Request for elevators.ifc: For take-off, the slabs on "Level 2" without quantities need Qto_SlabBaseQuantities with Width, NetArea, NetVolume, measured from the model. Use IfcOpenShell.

First a look at what the model holds.

```python
import ifcopenshell
import ifcopenshell.util.element
import ifcopenshell.util.unit

model = ifcopenshell.open("elevators.ifc")
print(model.schema)
for unit_type in ("LENGTHUNIT", "AREAUNIT", "VOLUMEUNIT"):
    print(unit_type, ifcopenshell.util.unit.calculate_unit_scale(model, unit_type))
storey = next(s for s in model.by_type("IfcBuildingStorey") if s.Name == "Level 2")
slabs = [e for e in ifcopenshell.util.element.get_decomposition(storey) if e.is_a("IfcSlab")]
for e in sorted(slabs, key=lambda e: e.id()):
    print(e.id(), e.is_a(), e.Name, list(ifcopenshell.util.element.get_psets(e, qtos_only=True)), sep=" | ")
```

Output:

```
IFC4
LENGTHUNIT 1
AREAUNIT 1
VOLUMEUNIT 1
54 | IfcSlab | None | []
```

```python
import ifcopenshell
import ifcopenshell.api.pset
import ifcopenshell.geom
import ifcopenshell.util.element
import ifcopenshell.util.shape
import ifcopenshell.util.unit

model = ifcopenshell.open("elevators.ifc")
unit_scale = ifcopenshell.util.unit.calculate_unit_scale(model)
area_scale = ifcopenshell.util.unit.calculate_unit_scale(model, "AREAUNIT")
volume_scale = ifcopenshell.util.unit.calculate_unit_scale(model, "VOLUMEUNIT")
settings = ifcopenshell.geom.settings()

storey = next(s for s in model.by_type("IfcBuildingStorey") if s.Name == "Level 2")
slabs = [e for e in ifcopenshell.util.element.get_decomposition(storey) if e.is_a("IfcSlab")]

for e in sorted(slabs, key=lambda e: e.id()):
    if ifcopenshell.util.element.get_psets(e, qtos_only=True, should_inherit=False):
        continue
    # Geometry comes back in metres, in the element's own axes.
    shape = ifcopenshell.geom.create_shape(settings, e)
    values = {
        "Width": ifcopenshell.util.shape.get_z(shape.geometry) / unit_scale,
        "NetArea": ifcopenshell.util.shape.get_footprint_area(shape.geometry) / area_scale,
        "NetVolume": ifcopenshell.util.shape.get_volume(shape.geometry) / volume_scale,
    }
    qto = ifcopenshell.api.pset.add_qto(model, product=e, name="Qto_SlabBaseQuantities")
    ifcopenshell.api.pset.edit_qto(model, qto=qto, properties=values)
    print(e.id(), {k: round(v, 3) for k, v in values.items()})

model.write("elevators_edited.ifc")
```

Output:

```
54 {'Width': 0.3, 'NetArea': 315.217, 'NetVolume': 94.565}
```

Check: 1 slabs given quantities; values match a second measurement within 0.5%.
